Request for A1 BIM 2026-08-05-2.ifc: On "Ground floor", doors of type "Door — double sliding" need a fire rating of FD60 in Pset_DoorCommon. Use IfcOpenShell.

First a look at what the model holds.

```python
import ifcopenshell
import ifcopenshell.util.element

model = ifcopenshell.open("A1 BIM 2026-08-05-2.ifc")
print(model.schema)
storey = next(s for s in model.by_type("IfcBuildingStorey") if s.Name == "Ground floor")
doors = [e for e in ifcopenshell.util.element.get_decomposition(storey) if e.is_a("IfcDoor")]
seen = {}
for e in doors:
    element_type = ifcopenshell.util.element.get_type(e)
    key = (element_type.Name if element_type != e and element_type else None, ifcopenshell.util.element.get_pset(e, "Pset_DoorCommon", "FireRating"))
    seen[key] = seen.get(key, 0) + 1
for (name, value), count in sorted(seen.items(), key=str):
    print(count, "x", name, "|", value)
```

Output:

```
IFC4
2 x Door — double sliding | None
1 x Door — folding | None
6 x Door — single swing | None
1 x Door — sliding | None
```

```python
import ifcopenshell
import ifcopenshell.api.pset
import ifcopenshell.util.element

model = ifcopenshell.open("A1 BIM 2026-08-05-2.ifc")

storey = next(s for s in model.by_type("IfcBuildingStorey") if s.Name == "Ground floor")
doors = [e for e in ifcopenshell.util.element.get_decomposition(storey) if e.is_a("IfcDoor")]

count = 0
for e in doors:
    element_type = ifcopenshell.util.element.get_type(e)
    if element_type in (None, e) or element_type.Name != "Door — double sliding":
        continue
    # add_pset returns the element's existing set when there is one.
    pset = ifcopenshell.api.pset.add_pset(model, product=e, name="Pset_DoorCommon")
    ifcopenshell.api.pset.edit_pset(model, pset=pset, properties={"FireRating": "FD60"})
    count += 1

print(count, "doors updated")

model.write("A1 BIM 2026-08-05-2_v2.ifc")
```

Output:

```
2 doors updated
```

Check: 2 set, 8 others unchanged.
